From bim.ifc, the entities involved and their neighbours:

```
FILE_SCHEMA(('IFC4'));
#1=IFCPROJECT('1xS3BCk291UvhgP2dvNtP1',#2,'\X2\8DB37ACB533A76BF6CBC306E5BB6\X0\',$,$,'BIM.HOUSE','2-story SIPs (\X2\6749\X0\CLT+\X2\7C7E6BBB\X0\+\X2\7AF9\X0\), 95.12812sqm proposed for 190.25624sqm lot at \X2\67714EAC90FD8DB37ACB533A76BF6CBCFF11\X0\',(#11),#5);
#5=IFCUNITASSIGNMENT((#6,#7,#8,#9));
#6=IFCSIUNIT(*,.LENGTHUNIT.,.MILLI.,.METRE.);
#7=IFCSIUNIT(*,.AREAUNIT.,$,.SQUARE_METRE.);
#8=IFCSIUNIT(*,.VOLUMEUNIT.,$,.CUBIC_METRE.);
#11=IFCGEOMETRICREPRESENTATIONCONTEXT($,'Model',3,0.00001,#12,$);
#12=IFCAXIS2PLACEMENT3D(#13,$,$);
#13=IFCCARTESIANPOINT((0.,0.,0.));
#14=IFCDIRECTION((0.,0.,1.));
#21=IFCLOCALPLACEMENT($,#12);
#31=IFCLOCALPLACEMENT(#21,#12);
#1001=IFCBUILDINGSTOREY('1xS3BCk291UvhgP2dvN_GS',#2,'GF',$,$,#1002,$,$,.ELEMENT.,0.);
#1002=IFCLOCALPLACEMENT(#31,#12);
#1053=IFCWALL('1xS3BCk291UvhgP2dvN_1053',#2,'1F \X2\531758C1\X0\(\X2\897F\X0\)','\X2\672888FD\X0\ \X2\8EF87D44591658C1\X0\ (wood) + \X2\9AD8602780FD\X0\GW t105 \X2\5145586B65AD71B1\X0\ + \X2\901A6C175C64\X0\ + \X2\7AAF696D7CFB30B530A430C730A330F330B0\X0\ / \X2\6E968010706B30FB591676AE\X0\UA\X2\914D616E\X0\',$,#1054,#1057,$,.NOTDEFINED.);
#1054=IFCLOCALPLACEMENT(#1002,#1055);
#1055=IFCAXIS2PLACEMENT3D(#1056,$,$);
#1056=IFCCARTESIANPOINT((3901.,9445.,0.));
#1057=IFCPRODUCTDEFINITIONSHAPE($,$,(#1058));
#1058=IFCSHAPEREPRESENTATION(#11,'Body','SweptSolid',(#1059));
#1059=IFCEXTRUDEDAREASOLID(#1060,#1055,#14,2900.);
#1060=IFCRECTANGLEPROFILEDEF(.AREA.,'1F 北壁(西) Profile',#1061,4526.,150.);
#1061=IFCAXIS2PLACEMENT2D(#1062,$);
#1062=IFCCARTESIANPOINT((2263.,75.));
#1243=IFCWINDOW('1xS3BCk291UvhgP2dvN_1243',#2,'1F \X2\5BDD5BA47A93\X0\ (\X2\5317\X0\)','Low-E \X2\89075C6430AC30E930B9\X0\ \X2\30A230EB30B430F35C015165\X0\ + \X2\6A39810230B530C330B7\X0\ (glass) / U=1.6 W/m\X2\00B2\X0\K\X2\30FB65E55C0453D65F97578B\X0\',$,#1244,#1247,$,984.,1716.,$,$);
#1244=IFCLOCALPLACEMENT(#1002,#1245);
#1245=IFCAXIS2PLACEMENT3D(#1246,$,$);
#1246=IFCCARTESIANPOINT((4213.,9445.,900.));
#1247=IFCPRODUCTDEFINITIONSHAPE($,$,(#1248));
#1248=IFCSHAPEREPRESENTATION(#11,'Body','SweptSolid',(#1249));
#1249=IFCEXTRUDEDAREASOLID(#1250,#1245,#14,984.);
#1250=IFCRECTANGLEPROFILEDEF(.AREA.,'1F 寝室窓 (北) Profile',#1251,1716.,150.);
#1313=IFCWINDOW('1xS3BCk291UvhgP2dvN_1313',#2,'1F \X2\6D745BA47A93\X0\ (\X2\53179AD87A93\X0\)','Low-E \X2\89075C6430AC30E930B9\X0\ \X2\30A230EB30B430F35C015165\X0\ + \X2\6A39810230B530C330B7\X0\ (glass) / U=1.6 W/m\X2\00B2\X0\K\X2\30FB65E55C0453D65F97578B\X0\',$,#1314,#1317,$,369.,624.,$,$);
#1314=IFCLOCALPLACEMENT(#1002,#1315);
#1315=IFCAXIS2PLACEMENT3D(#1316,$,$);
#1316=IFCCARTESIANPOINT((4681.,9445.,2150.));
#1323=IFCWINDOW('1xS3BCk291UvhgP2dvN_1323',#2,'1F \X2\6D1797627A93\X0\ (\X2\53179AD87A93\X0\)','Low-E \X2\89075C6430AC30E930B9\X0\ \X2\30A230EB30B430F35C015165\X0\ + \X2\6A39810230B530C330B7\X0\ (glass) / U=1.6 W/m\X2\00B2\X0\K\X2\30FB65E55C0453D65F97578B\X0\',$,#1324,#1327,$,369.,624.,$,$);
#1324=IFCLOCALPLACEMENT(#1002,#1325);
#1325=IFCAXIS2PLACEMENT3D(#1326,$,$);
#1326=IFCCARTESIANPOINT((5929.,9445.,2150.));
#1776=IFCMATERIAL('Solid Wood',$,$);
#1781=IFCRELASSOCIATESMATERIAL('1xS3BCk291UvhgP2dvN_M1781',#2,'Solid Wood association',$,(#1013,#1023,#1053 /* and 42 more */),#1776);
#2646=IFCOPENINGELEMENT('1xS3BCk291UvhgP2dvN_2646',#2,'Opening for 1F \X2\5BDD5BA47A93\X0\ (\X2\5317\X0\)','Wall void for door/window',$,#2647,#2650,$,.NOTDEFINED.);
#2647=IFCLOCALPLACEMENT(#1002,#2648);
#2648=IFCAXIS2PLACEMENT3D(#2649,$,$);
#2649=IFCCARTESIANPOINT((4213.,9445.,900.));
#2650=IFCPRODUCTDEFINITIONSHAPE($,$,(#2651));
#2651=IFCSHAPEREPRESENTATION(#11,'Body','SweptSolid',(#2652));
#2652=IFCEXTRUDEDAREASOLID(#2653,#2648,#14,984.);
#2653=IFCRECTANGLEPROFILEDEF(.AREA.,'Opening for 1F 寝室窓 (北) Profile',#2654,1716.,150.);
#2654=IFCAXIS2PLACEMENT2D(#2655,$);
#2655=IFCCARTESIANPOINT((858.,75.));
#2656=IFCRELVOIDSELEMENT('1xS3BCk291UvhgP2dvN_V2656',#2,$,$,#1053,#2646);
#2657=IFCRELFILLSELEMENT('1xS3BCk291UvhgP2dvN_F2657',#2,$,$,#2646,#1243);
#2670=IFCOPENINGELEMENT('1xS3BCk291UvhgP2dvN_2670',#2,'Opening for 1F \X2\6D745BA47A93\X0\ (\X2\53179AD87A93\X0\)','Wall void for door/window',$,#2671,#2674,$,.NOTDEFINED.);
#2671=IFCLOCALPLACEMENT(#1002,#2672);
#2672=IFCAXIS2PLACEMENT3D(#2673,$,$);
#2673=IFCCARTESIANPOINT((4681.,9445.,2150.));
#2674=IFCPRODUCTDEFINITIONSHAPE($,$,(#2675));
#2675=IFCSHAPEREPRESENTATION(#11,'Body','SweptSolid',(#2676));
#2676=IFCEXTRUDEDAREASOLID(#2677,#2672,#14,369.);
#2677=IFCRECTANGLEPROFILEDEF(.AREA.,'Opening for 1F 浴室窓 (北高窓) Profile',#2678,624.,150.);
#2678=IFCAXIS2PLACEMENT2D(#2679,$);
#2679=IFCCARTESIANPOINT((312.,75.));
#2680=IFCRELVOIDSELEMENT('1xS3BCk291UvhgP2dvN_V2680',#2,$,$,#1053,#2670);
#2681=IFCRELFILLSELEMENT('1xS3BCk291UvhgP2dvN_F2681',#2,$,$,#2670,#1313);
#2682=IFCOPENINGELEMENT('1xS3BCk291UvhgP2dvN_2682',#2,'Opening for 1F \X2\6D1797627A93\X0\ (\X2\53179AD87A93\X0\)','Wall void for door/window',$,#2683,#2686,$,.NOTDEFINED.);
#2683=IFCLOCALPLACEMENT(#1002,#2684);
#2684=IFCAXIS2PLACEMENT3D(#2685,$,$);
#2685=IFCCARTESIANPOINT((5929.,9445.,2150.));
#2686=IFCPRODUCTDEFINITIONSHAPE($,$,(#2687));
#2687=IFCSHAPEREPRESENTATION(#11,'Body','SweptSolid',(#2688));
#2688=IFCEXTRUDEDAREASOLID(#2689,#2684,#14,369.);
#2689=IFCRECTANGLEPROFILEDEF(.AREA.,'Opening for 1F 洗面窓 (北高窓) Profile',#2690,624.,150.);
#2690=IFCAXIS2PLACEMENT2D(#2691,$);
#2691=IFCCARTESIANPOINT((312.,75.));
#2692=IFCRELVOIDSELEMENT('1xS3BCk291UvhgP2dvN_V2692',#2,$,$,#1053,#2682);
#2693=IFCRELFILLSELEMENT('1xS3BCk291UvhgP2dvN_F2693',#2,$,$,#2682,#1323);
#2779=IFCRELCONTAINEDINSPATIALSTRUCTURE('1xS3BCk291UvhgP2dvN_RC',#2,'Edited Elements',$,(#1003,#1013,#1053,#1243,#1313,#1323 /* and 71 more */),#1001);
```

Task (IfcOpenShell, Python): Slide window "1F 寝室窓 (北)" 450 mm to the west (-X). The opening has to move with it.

```python
import ifcopenshell
import ifcopenshell.api.geometry
import ifcopenshell.util.placement

model = ifcopenshell.open("bim.ifc")

window = model.by_id(1243)
opening = window.FillsVoids[0].RelatingOpeningElement
wall = opening.VoidsElements[0].RelatingBuildingElement

wall_matrix = ifcopenshell.util.placement.get_local_placement(wall.ObjectPlacement)
shift = wall_matrix[:3, 0] * -450.0
before = ifcopenshell.util.placement.get_local_placement(window.ObjectPlacement)[:3, 3].copy()

# The window is not placed relative to its opening, so move both.
for product in (opening, window):
    matrix = ifcopenshell.util.placement.get_local_placement(product.ObjectPlacement)
    matrix[:3, 3] += shift
    ifcopenshell.api.geometry.edit_object_placement(model, product=product, matrix=matrix, is_si=False)

after = ifcopenshell.util.placement.get_local_placement(window.ObjectPlacement)[:3, 3]
print("window moved by", (after - before).round(3) + 0.0)

model.write("bim_v2.ifc")
```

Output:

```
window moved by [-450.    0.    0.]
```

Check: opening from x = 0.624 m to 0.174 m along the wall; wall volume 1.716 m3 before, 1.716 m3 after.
